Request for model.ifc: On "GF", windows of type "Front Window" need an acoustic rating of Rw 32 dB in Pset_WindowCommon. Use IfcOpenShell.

First a look at what the model holds.

```python
import ifcopenshell
import ifcopenshell.util.element

model = ifcopenshell.open("model.ifc")
print(model.schema)
storey = next(s for s in model.by_type("IfcBuildingStorey") if s.Name == "GF")
windows = [e for e in ifcopenshell.util.element.get_decomposition(storey) if e.is_a("IfcWindow")]
seen = {}
for e in windows:
    element_type = ifcopenshell.util.element.get_type(e)
    key = (element_type.Name if element_type != e and element_type else None, ifcopenshell.util.element.get_pset(e, "Pset_WindowCommon", "AcousticRating"))
    seen[key] = seen.get(key, 0) + 1
for (name, value), count in sorted(seen.items(), key=str):
    print(count, "x", name, "|", value)
```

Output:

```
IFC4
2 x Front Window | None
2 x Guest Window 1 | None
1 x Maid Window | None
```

```python
import ifcopenshell
import ifcopenshell.api.pset
import ifcopenshell.util.element

model = ifcopenshell.open("model.ifc")

storey = next(s for s in model.by_type("IfcBuildingStorey") if s.Name == "GF")
windows = [e for e in ifcopenshell.util.element.get_decomposition(storey) if e.is_a("IfcWindow")]

count = 0
for e in windows:
    element_type = ifcopenshell.util.element.get_type(e)
    if element_type in (None, e) or element_type.Name != "Front Window":
        continue
    # add_pset returns the element's existing set when there is one.
    pset = ifcopenshell.api.pset.add_pset(model, product=e, name="Pset_WindowCommon")
    ifcopenshell.api.pset.edit_pset(model, pset=pset, properties={"AcousticRating": "Rw 32 dB"})
    count += 1

print(count, "windows updated")

model.write("model_edited.ifc")
```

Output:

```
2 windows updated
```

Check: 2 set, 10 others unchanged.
